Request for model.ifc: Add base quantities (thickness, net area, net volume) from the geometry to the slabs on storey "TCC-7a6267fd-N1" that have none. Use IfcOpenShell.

First a look at what the model holds.

```python
import ifcopenshell
import ifcopenshell.util.element
import ifcopenshell.util.unit

model = ifcopenshell.open("model.ifc")
print(model.schema)
for unit_type in ("LENGTHUNIT", "AREAUNIT", "VOLUMEUNIT"):
    print(unit_type, ifcopenshell.util.unit.calculate_unit_scale(model, unit_type))
storey = next(s for s in model.by_type("IfcBuildingStorey") if s.Name == "TCC-7a6267fd-N1")
slabs = [e for e in ifcopenshell.util.element.get_decomposition(storey) if e.is_a("IfcSlab")]
for e in sorted(slabs, key=lambda e: e.id()):
    print(e.id(), e.is_a(), e.Name, list(ifcopenshell.util.element.get_psets(e, qtos_only=True)), sep=" | ")
```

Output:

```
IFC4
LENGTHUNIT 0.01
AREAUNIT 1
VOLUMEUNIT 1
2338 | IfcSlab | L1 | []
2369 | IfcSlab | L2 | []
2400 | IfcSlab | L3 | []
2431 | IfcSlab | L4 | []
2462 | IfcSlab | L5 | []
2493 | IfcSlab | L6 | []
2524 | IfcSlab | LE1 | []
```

```python
import ifcopenshell
import ifcopenshell.api.pset
import ifcopenshell.geom
import ifcopenshell.util.element
import ifcopenshell.util.shape
import ifcopenshell.util.unit

model = ifcopenshell.open("model.ifc")
unit_scale = ifcopenshell.util.unit.calculate_unit_scale(model)
area_scale = ifcopenshell.util.unit.calculate_unit_scale(model, "AREAUNIT")
volume_scale = ifcopenshell.util.unit.calculate_unit_scale(model, "VOLUMEUNIT")
settings = ifcopenshell.geom.settings()

storey = next(s for s in model.by_type("IfcBuildingStorey") if s.Name == "TCC-7a6267fd-N1")
slabs = [e for e in ifcopenshell.util.element.get_decomposition(storey) if e.is_a("IfcSlab")]

for e in sorted(slabs, key=lambda e: e.id()):
    if ifcopenshell.util.element.get_psets(e, qtos_only=True, should_inherit=False):
        continue
    # Geometry comes back in metres, in the element's own axes.
    shape = ifcopenshell.geom.create_shape(settings, e)
    values = {
        "Width": ifcopenshell.util.shape.get_z(shape.geometry) / unit_scale,
        "NetArea": ifcopenshell.util.shape.get_footprint_area(shape.geometry) / area_scale,
        "NetVolume": ifcopenshell.util.shape.get_volume(shape.geometry) / volume_scale,
    }
    qto = ifcopenshell.api.pset.add_qto(model, product=e, name="Qto_SlabBaseQuantities")
    ifcopenshell.api.pset.edit_qto(model, qto=qto, properties=values)
    print(e.id(), {k: round(v, 3) for k, v in values.items()})

model.write("model_rev.ifc")
```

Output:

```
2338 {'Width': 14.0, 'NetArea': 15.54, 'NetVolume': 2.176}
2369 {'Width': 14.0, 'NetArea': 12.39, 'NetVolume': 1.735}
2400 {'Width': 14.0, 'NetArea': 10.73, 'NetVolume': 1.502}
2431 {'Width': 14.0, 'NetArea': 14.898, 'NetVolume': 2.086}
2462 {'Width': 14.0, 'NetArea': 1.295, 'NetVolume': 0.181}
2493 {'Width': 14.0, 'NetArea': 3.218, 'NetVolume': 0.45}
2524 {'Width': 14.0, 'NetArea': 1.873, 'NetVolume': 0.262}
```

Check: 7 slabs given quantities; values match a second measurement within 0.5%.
